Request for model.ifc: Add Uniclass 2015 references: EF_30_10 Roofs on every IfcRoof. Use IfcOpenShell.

First a look at what the model holds.

```python
import ifcopenshell

model = ifcopenshell.open("model.ifc")
print(model.schema)
print("classifications:", [c.Name for c in model.by_type("IfcClassification")])
for ifc_class in ("IfcDoor", "IfcRoof", "IfcStair", "IfcWall", "IfcWindow"):
    print(ifc_class, len(model.by_type(ifc_class)))
```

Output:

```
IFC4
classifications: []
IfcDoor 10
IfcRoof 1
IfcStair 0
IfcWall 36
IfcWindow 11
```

```python
import ifcopenshell
import ifcopenshell.api.classification

model = ifcopenshell.open("model.ifc")

system = ifcopenshell.api.classification.add_classification(model, classification="Uniclass 2015")

codes = {
    "IfcRoof": ("EF_30_10", "Roofs"),
}
for ifc_class, (code, name) in codes.items():
    products = model.by_type(ifc_class)
    ifcopenshell.api.classification.add_reference(
        model, products=products, classification=system, identification=code, name=name
    )
    print(code, len(products))

model.write("model_updated.ifc")
```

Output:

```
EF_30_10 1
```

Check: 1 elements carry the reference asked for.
